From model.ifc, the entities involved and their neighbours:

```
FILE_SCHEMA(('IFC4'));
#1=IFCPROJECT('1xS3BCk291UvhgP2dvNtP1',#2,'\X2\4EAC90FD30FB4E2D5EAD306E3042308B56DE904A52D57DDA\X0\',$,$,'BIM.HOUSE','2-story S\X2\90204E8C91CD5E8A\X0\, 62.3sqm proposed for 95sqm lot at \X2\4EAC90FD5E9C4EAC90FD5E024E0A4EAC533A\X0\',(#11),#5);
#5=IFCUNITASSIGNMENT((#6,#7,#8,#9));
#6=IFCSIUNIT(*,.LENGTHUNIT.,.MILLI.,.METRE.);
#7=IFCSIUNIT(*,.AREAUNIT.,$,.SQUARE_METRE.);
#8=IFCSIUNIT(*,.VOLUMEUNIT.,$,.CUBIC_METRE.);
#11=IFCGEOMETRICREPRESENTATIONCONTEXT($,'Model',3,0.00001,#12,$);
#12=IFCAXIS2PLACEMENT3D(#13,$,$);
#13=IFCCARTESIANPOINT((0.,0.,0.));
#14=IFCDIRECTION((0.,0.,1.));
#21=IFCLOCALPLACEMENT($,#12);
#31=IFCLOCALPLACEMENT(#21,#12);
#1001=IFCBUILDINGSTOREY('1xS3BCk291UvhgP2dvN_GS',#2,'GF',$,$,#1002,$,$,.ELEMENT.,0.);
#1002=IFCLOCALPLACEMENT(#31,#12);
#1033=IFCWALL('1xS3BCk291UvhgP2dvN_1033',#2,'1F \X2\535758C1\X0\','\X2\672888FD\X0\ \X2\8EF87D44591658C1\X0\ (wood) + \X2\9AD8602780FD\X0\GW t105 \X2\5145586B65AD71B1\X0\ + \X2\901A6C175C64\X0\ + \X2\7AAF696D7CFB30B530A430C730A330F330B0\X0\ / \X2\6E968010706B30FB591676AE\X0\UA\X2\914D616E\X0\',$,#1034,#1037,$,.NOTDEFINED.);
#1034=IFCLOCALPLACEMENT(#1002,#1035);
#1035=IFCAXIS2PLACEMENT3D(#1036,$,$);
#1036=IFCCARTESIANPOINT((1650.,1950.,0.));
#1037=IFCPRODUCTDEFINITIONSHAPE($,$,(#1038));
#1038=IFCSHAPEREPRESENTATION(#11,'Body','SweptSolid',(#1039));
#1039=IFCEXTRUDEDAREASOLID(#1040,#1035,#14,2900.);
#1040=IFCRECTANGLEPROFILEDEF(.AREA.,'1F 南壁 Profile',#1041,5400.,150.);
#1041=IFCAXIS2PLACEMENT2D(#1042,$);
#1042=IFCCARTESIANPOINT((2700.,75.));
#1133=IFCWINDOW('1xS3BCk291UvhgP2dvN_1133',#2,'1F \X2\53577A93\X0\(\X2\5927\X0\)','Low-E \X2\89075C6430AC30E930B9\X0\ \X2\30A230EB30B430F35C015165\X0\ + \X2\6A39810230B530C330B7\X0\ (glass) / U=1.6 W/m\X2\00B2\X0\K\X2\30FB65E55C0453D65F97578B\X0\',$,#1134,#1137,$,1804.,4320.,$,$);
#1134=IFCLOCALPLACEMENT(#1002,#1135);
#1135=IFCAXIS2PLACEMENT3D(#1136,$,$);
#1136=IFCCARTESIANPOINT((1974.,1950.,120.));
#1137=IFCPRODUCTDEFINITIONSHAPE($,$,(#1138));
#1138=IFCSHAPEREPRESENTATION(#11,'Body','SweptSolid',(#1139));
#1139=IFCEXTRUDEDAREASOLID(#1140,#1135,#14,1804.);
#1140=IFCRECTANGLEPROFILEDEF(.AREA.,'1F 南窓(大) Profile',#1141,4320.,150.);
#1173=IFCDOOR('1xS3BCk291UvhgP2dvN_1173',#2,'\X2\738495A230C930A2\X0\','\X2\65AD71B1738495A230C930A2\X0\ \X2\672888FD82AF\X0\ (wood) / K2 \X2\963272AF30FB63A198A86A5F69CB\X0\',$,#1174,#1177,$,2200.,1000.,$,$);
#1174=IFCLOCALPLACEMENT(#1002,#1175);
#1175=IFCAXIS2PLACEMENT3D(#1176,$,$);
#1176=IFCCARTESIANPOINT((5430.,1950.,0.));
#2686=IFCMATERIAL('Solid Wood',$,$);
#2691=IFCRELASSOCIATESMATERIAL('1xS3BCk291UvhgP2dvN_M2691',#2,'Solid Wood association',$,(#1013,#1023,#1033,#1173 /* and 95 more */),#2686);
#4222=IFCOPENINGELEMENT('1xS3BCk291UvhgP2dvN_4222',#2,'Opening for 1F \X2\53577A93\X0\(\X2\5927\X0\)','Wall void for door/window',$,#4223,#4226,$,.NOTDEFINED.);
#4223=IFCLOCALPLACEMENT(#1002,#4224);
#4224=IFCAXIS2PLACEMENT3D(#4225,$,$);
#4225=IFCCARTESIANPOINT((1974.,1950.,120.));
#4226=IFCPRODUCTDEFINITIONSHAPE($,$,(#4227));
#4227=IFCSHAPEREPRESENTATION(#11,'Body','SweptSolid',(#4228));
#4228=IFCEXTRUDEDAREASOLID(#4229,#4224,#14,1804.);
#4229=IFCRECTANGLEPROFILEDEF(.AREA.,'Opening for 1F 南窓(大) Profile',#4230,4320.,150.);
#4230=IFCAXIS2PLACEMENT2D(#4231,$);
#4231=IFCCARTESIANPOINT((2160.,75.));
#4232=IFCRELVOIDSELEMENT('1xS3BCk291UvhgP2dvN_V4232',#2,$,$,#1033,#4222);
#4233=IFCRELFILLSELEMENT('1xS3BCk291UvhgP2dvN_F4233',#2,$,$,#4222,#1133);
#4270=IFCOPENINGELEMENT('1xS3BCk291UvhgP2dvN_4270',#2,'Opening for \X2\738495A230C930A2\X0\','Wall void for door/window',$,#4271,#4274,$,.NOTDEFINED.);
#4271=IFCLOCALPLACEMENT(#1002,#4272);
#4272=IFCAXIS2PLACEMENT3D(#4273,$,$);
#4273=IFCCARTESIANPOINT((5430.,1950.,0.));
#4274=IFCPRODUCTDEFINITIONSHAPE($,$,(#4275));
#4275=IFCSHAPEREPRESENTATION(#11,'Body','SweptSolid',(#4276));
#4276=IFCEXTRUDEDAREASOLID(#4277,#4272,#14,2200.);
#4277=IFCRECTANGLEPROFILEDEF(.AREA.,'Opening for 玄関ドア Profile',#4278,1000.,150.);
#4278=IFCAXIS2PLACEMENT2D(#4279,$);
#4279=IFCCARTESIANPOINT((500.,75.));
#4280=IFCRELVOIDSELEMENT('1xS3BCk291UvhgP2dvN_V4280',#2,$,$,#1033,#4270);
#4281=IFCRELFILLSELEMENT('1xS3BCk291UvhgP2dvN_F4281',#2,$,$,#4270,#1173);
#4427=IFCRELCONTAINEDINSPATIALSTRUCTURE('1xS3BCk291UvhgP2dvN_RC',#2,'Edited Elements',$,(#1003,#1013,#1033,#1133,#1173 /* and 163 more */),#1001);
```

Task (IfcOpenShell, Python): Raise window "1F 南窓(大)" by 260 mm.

```python
import numpy as np
import ifcopenshell
import ifcopenshell.api.geometry
import ifcopenshell.util.placement
import ifcopenshell.util.unit

model = ifcopenshell.open("model.ifc")
unit_scale = ifcopenshell.util.unit.calculate_unit_scale(model)

window = model.by_guid("1xS3BCk291UvhgP2dvN_1133")
opening = window.FillsVoids[0].RelatingOpeningElement
dz = 260.0

shift = np.array([0.0, 0.0, dz])
# The window is not placed relative to its opening, so move both.
for product in (opening, window):
    matrix = ifcopenshell.util.placement.get_local_placement(product.ObjectPlacement)
    matrix[:3, 3] += shift
    ifcopenshell.api.geometry.edit_object_placement(model, product=product, matrix=matrix, is_si=False)

print(f"moved by {dz * unit_scale:+.3f} m")

model.write("model_rev.ifc")
```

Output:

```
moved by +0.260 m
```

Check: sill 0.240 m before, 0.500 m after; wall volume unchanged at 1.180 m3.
